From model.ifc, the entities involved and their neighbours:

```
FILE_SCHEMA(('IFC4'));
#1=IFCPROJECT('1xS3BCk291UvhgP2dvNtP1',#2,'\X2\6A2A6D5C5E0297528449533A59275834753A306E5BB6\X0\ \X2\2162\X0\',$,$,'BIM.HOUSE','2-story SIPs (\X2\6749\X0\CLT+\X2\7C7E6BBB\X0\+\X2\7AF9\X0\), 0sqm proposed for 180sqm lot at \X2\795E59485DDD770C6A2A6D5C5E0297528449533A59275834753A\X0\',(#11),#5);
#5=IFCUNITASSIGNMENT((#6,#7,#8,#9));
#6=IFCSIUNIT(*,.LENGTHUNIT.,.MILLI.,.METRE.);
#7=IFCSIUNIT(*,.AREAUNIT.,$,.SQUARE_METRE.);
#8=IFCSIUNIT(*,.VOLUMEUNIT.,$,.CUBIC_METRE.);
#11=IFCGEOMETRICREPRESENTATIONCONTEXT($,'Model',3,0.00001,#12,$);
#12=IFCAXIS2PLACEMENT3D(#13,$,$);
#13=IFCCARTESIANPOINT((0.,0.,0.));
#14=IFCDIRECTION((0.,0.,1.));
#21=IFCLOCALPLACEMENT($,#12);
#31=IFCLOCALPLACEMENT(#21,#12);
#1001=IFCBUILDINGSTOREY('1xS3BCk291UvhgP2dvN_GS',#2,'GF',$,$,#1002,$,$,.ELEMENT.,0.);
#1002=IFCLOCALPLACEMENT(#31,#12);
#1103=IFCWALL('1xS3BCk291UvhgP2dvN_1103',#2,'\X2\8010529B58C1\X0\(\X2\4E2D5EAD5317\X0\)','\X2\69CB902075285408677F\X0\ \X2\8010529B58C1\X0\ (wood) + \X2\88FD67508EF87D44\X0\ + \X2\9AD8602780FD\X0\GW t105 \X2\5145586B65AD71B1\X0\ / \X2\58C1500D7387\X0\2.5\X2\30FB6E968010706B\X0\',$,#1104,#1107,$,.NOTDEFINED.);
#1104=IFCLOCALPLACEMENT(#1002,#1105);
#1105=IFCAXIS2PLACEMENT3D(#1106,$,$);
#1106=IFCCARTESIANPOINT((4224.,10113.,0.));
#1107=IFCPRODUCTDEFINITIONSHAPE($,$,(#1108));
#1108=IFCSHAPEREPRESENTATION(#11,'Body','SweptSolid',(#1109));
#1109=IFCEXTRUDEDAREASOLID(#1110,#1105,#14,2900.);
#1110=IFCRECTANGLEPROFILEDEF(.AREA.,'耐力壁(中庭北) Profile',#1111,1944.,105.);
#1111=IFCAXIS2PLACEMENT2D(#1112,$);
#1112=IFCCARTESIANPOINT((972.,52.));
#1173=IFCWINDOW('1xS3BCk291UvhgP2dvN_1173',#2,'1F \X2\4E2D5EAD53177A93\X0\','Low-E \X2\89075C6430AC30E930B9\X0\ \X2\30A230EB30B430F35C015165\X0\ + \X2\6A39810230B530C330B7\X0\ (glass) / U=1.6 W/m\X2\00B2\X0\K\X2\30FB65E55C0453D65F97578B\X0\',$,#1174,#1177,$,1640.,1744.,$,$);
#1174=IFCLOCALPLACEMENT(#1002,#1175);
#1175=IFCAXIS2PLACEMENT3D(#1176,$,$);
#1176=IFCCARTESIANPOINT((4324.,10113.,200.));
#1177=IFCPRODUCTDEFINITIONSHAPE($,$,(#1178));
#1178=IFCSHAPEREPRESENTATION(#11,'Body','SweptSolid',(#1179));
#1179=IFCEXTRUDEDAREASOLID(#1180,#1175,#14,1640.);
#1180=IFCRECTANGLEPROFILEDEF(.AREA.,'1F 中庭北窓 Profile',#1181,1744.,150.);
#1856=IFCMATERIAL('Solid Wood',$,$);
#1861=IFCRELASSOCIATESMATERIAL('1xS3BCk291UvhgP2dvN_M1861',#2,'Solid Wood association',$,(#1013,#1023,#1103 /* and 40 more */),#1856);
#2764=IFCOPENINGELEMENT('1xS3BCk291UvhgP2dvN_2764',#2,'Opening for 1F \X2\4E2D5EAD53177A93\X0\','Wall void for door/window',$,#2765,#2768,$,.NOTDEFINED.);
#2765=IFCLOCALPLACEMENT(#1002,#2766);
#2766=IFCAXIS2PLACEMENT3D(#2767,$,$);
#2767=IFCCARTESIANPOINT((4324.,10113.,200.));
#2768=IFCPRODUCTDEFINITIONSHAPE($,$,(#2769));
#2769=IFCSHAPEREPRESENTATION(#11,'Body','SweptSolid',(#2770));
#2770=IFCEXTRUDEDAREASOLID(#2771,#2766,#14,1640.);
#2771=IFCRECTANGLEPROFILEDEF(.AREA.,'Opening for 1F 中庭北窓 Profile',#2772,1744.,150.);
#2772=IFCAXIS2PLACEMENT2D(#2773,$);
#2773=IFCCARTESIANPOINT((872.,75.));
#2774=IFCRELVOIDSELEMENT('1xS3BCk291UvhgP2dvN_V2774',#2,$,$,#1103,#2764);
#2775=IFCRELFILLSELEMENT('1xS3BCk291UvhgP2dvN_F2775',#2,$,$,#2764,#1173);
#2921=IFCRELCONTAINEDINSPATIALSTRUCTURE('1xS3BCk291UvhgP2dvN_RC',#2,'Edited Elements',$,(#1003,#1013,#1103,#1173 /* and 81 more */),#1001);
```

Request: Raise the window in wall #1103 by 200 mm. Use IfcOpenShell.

```python
import numpy as np
import ifcopenshell
import ifcopenshell.api.geometry
import ifcopenshell.util.placement
import ifcopenshell.util.unit

model = ifcopenshell.open("model.ifc")
unit_scale = ifcopenshell.util.unit.calculate_unit_scale(model)

window = model.by_guid("1xS3BCk291UvhgP2dvN_1173")
opening = window.FillsVoids[0].RelatingOpeningElement
dz = 200.0

shift = np.array([0.0, 0.0, dz])
# The window is not placed relative to its opening, so move both.
for product in (opening, window):
    matrix = ifcopenshell.util.placement.get_local_placement(product.ObjectPlacement)
    matrix[:3, 3] += shift
    ifcopenshell.api.geometry.edit_object_placement(model, product=product, matrix=matrix, is_si=False)

print(f"moved by {dz * unit_scale:+.3f} m")

model.write("model_updated.ifc")
```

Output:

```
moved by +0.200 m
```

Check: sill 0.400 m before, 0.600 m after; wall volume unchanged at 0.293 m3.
